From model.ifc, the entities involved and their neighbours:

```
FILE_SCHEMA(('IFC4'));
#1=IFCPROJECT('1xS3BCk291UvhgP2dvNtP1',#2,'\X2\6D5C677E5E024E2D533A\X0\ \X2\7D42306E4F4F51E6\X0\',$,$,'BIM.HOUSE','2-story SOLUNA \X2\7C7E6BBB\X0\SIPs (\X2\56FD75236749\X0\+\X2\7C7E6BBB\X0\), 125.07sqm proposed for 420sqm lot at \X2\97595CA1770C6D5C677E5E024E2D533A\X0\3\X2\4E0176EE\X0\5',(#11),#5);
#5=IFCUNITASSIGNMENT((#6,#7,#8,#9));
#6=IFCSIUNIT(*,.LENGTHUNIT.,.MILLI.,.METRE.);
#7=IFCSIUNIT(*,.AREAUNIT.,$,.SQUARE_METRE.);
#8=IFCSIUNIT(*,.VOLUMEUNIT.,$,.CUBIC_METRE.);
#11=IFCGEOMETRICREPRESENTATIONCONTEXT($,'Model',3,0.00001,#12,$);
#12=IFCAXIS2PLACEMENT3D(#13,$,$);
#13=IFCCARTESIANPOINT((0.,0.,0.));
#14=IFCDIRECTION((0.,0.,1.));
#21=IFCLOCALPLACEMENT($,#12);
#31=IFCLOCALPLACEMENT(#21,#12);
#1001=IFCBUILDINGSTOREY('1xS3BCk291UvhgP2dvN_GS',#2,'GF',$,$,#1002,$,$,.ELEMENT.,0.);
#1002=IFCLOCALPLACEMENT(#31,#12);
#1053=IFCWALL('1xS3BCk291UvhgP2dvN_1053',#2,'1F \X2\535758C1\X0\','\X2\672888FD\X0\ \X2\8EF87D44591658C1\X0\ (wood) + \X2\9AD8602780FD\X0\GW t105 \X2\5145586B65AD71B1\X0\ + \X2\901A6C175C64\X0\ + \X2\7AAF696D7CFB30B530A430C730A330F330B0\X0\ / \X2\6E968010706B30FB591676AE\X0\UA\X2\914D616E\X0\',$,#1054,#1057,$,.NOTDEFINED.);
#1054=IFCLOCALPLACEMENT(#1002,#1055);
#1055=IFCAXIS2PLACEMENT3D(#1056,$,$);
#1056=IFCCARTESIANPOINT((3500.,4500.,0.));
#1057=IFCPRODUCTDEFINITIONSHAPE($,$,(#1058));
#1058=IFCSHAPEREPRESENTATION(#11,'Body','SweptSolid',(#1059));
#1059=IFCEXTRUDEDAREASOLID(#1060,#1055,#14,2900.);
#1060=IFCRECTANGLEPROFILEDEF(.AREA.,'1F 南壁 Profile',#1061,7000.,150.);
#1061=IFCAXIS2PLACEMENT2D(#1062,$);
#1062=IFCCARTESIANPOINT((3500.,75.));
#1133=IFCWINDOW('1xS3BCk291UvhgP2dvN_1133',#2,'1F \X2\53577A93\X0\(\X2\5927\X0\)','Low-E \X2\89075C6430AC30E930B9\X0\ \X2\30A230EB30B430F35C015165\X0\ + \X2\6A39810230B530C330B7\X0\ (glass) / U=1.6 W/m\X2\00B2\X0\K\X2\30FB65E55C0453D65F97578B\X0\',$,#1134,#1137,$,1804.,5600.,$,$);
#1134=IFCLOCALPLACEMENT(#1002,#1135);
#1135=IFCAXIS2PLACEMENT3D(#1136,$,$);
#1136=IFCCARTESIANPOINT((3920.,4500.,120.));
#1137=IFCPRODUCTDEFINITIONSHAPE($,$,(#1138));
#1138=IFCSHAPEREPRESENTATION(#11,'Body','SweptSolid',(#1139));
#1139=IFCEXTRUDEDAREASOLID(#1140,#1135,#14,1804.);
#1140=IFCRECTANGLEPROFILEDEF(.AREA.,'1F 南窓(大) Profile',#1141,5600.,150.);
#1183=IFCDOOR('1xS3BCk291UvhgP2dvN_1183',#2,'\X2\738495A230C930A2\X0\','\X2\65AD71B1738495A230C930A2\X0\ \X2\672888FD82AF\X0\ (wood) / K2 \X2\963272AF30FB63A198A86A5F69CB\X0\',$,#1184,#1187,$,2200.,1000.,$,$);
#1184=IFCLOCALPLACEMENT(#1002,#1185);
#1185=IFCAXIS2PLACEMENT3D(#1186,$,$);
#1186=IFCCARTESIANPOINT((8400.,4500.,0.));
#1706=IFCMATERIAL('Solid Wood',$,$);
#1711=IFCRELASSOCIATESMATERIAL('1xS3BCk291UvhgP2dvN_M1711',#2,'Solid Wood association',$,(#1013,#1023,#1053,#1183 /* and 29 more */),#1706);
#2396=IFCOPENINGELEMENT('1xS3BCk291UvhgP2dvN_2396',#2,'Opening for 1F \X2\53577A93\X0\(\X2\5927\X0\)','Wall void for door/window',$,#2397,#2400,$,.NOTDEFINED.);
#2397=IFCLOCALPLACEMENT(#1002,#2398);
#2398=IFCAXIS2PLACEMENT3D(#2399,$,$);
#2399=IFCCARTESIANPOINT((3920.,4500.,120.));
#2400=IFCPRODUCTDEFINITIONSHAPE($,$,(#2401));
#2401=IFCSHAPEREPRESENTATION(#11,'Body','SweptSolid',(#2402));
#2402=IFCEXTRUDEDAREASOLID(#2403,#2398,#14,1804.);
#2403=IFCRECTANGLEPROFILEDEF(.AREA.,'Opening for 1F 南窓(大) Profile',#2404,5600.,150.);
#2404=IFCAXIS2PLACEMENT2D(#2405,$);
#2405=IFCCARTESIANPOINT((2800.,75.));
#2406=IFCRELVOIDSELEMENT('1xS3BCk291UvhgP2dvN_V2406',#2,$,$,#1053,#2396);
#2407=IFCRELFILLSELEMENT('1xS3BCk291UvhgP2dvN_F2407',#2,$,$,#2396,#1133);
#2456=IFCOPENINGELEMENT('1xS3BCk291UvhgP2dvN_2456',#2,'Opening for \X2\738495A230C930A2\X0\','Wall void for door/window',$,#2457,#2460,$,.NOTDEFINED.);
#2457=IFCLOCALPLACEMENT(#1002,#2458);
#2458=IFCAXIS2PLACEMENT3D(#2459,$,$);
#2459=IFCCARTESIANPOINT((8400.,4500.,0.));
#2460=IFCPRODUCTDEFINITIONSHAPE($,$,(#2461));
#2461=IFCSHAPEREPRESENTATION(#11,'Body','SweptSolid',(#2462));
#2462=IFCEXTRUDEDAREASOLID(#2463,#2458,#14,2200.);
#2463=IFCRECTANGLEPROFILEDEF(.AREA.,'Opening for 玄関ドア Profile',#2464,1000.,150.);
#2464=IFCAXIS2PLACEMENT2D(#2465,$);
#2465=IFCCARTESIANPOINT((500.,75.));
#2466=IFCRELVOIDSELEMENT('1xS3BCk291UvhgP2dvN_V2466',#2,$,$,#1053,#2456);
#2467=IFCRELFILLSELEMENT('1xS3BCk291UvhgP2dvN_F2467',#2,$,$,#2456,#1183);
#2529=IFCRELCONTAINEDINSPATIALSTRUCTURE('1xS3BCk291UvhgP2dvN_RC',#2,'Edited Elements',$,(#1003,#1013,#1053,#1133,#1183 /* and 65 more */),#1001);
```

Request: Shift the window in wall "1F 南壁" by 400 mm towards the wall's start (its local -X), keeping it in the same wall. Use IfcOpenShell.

```python
import ifcopenshell
import ifcopenshell.api.geometry
import ifcopenshell.util.placement

model = ifcopenshell.open("model.ifc")

window = model.by_guid("1xS3BCk291UvhgP2dvN_1133")
opening = window.FillsVoids[0].RelatingOpeningElement
wall = opening.VoidsElements[0].RelatingBuildingElement

wall_matrix = ifcopenshell.util.placement.get_local_placement(wall.ObjectPlacement)
shift = wall_matrix[:3, 0] * -400.0
before = ifcopenshell.util.placement.get_local_placement(window.ObjectPlacement)[:3, 3].copy()

# The window is not placed relative to its opening, so move both.
for product in (opening, window):
    matrix = ifcopenshell.util.placement.get_local_placement(product.ObjectPlacement)
    matrix[:3, 3] += shift
    ifcopenshell.api.geometry.edit_object_placement(model, product=product, matrix=matrix, is_si=False)

after = ifcopenshell.util.placement.get_local_placement(window.ObjectPlacement)[:3, 3]
print("window moved by", (after - before).round(3) + 0.0)

model.write("model_rev.ifc")
```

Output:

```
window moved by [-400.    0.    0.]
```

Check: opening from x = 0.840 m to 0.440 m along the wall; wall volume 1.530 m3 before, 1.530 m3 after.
